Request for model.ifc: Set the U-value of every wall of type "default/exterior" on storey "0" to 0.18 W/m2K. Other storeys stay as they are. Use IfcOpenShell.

First a look at what the model holds.

```python
import ifcopenshell
import ifcopenshell.util.element

model = ifcopenshell.open("model.ifc")
print(model.schema)
storey = next(s for s in model.by_type("IfcBuildingStorey") if s.Name == "0")
walls = [e for e in ifcopenshell.util.element.get_decomposition(storey) if e.is_a("IfcWall")]
seen = {}
for e in walls:
    element_type = ifcopenshell.util.element.get_type(e)
    key = (element_type.Name if element_type != e and element_type else None, ifcopenshell.util.element.get_pset(e, "Pset_WallCommon", "ThermalTransmittance"))
    seen[key] = seen.get(key, 0) + 1
for (name, value), count in sorted(seen.items(), key=str):
    print(count, "x", name, "|", value)
```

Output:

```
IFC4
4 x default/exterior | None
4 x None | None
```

```python
import ifcopenshell
import ifcopenshell.api.pset
import ifcopenshell.util.element

model = ifcopenshell.open("model.ifc")

storey = next(s for s in model.by_type("IfcBuildingStorey") if s.Name == "0")
walls = [e for e in ifcopenshell.util.element.get_decomposition(storey) if e.is_a("IfcWall")]

count = 0
for e in walls:
    element_type = ifcopenshell.util.element.get_type(e)
    if element_type in (None, e) or element_type.Name != "default/exterior":
        continue
    # add_pset returns the element's existing set when there is one.
    pset = ifcopenshell.api.pset.add_pset(model, product=e, name="Pset_WallCommon")
    ifcopenshell.api.pset.edit_pset(model, pset=pset, properties={"ThermalTransmittance": 0.18})
    count += 1

print(count, "walls updated")

model.write("model_edited.ifc")
```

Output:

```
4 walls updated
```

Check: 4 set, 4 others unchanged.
